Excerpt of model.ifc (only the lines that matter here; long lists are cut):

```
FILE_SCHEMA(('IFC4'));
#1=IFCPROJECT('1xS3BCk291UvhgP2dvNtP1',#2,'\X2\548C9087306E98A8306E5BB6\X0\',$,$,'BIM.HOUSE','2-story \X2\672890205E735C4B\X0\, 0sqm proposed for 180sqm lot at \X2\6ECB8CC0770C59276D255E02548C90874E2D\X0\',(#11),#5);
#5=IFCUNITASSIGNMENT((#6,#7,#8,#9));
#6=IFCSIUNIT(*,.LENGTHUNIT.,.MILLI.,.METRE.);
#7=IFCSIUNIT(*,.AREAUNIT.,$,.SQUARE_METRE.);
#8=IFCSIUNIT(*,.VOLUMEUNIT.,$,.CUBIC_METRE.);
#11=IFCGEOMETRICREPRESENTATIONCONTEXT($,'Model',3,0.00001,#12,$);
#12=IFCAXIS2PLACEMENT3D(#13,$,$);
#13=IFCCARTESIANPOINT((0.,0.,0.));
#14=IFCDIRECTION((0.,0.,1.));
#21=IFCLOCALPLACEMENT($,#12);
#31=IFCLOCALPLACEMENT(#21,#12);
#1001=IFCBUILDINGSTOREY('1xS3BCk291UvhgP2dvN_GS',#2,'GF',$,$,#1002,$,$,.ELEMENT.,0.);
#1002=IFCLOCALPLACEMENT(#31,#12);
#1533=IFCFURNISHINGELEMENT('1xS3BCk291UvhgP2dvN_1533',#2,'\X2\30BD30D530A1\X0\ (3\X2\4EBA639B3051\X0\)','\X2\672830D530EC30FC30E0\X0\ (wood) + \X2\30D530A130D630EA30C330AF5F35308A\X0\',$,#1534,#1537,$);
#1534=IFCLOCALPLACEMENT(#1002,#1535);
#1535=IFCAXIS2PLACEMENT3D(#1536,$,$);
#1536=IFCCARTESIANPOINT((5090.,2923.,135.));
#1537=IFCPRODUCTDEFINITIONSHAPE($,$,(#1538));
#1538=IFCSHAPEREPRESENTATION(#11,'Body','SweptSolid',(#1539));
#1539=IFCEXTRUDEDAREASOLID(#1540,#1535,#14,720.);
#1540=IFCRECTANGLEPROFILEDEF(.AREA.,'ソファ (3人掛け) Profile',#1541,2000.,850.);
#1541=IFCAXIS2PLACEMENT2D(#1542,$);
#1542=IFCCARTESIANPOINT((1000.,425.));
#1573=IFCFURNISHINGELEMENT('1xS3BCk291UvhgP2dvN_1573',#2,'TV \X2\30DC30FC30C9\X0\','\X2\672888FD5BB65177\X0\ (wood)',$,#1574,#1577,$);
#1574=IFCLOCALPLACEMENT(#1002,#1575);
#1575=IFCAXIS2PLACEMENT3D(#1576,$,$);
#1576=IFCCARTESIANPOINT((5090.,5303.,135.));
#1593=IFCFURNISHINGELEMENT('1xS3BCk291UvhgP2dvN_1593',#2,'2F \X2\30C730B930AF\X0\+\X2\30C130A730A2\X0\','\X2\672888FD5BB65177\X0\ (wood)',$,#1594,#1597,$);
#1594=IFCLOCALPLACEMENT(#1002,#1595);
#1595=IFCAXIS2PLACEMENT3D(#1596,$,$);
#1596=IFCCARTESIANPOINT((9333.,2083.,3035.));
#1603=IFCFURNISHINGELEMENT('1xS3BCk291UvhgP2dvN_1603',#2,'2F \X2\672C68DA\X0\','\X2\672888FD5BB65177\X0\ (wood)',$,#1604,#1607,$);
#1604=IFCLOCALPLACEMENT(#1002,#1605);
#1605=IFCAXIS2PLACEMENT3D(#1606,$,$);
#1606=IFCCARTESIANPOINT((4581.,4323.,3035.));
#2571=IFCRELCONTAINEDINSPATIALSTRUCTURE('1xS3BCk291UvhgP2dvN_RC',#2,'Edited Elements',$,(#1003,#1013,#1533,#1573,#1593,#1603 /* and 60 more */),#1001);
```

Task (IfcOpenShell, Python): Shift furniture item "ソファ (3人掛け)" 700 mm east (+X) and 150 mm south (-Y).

```python
import ifcopenshell
import ifcopenshell.api.geometry
import ifcopenshell.util.placement
import ifcopenshell.util.unit

model = ifcopenshell.open("model.ifc")
unit_scale = ifcopenshell.util.unit.calculate_unit_scale(model)

item = model.by_id(1533)
matrix = ifcopenshell.util.placement.get_local_placement(item.ObjectPlacement)
matrix[0, 3] += 0.7 / unit_scale
matrix[1, 3] -= 0.15 / unit_scale
ifcopenshell.api.geometry.edit_object_placement(model, product=item, matrix=matrix, is_si=False)

print(ifcopenshell.util.placement.get_local_placement(item.ObjectPlacement).round(3) + 0.0)

model.write("model-out.ifc")
```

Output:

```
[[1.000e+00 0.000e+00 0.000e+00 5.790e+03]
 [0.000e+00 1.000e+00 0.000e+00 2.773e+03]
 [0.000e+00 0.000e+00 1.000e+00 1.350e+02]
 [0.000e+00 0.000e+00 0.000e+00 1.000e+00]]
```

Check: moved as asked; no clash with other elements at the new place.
